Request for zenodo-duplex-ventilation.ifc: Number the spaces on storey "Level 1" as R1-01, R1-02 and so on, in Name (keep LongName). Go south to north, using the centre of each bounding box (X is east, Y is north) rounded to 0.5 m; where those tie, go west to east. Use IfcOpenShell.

First a look at what the model holds.

```python
import ifcopenshell
import ifcopenshell.util.element
import ifcopenshell.util.placement

model = ifcopenshell.open("zenodo-duplex-ventilation.ifc")
print(model.schema)
storey = next(s for s in model.by_type("IfcBuildingStorey") if s.Name == "Level 1")
spaces = [e for e in ifcopenshell.util.element.get_decomposition(storey) if e.is_a("IfcSpace")]
for e in sorted(spaces, key=lambda e: e.id()):
    origin = ifcopenshell.util.placement.get_local_placement(e.ObjectPlacement)[:3, 3]
    print(e.id(), e.Name, e.LongName, origin.round(2) + 0.0, sep=" | ")
```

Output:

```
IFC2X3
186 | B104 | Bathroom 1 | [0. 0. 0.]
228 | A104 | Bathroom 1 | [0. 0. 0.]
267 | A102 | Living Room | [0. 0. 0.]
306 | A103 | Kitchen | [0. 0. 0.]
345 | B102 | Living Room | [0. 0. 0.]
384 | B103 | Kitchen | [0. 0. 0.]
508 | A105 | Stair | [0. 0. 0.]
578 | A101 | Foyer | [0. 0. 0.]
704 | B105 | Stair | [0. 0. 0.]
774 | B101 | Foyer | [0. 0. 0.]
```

```python
import ifcopenshell
import ifcopenshell.geom
import ifcopenshell.util.element
import ifcopenshell.util.shape

model = ifcopenshell.open("zenodo-duplex-ventilation.ifc")
settings = ifcopenshell.geom.settings()
settings.set("use-world-coords", True)


def centre(element):
    shape = ifcopenshell.geom.create_shape(settings, element)
    return ifcopenshell.util.shape.get_bbox_centroid(shape.geometry)


storey = next(s for s in model.by_type("IfcBuildingStorey") if s.Name == "Level 1")
spaces = [e for e in ifcopenshell.util.element.get_decomposition(storey) if e.is_a("IfcSpace")]

# Insertion points can sit at a corner or the storey origin, so sort by the geometry (in metres).
centres = {e: centre(e) for e in spaces}
spaces.sort(key=lambda e: (round(centres[e][1] / 0.5), centres[e][0]))

for i, e in enumerate(spaces, start=1):
    number = f"R1-{i:02d}"
    e.Name = number
    print(e.id(), number)

model.write("zenodo-duplex-ventilation_v2.ifc")
```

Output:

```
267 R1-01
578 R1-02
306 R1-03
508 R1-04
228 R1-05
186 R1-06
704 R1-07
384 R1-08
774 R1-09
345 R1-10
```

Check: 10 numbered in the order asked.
